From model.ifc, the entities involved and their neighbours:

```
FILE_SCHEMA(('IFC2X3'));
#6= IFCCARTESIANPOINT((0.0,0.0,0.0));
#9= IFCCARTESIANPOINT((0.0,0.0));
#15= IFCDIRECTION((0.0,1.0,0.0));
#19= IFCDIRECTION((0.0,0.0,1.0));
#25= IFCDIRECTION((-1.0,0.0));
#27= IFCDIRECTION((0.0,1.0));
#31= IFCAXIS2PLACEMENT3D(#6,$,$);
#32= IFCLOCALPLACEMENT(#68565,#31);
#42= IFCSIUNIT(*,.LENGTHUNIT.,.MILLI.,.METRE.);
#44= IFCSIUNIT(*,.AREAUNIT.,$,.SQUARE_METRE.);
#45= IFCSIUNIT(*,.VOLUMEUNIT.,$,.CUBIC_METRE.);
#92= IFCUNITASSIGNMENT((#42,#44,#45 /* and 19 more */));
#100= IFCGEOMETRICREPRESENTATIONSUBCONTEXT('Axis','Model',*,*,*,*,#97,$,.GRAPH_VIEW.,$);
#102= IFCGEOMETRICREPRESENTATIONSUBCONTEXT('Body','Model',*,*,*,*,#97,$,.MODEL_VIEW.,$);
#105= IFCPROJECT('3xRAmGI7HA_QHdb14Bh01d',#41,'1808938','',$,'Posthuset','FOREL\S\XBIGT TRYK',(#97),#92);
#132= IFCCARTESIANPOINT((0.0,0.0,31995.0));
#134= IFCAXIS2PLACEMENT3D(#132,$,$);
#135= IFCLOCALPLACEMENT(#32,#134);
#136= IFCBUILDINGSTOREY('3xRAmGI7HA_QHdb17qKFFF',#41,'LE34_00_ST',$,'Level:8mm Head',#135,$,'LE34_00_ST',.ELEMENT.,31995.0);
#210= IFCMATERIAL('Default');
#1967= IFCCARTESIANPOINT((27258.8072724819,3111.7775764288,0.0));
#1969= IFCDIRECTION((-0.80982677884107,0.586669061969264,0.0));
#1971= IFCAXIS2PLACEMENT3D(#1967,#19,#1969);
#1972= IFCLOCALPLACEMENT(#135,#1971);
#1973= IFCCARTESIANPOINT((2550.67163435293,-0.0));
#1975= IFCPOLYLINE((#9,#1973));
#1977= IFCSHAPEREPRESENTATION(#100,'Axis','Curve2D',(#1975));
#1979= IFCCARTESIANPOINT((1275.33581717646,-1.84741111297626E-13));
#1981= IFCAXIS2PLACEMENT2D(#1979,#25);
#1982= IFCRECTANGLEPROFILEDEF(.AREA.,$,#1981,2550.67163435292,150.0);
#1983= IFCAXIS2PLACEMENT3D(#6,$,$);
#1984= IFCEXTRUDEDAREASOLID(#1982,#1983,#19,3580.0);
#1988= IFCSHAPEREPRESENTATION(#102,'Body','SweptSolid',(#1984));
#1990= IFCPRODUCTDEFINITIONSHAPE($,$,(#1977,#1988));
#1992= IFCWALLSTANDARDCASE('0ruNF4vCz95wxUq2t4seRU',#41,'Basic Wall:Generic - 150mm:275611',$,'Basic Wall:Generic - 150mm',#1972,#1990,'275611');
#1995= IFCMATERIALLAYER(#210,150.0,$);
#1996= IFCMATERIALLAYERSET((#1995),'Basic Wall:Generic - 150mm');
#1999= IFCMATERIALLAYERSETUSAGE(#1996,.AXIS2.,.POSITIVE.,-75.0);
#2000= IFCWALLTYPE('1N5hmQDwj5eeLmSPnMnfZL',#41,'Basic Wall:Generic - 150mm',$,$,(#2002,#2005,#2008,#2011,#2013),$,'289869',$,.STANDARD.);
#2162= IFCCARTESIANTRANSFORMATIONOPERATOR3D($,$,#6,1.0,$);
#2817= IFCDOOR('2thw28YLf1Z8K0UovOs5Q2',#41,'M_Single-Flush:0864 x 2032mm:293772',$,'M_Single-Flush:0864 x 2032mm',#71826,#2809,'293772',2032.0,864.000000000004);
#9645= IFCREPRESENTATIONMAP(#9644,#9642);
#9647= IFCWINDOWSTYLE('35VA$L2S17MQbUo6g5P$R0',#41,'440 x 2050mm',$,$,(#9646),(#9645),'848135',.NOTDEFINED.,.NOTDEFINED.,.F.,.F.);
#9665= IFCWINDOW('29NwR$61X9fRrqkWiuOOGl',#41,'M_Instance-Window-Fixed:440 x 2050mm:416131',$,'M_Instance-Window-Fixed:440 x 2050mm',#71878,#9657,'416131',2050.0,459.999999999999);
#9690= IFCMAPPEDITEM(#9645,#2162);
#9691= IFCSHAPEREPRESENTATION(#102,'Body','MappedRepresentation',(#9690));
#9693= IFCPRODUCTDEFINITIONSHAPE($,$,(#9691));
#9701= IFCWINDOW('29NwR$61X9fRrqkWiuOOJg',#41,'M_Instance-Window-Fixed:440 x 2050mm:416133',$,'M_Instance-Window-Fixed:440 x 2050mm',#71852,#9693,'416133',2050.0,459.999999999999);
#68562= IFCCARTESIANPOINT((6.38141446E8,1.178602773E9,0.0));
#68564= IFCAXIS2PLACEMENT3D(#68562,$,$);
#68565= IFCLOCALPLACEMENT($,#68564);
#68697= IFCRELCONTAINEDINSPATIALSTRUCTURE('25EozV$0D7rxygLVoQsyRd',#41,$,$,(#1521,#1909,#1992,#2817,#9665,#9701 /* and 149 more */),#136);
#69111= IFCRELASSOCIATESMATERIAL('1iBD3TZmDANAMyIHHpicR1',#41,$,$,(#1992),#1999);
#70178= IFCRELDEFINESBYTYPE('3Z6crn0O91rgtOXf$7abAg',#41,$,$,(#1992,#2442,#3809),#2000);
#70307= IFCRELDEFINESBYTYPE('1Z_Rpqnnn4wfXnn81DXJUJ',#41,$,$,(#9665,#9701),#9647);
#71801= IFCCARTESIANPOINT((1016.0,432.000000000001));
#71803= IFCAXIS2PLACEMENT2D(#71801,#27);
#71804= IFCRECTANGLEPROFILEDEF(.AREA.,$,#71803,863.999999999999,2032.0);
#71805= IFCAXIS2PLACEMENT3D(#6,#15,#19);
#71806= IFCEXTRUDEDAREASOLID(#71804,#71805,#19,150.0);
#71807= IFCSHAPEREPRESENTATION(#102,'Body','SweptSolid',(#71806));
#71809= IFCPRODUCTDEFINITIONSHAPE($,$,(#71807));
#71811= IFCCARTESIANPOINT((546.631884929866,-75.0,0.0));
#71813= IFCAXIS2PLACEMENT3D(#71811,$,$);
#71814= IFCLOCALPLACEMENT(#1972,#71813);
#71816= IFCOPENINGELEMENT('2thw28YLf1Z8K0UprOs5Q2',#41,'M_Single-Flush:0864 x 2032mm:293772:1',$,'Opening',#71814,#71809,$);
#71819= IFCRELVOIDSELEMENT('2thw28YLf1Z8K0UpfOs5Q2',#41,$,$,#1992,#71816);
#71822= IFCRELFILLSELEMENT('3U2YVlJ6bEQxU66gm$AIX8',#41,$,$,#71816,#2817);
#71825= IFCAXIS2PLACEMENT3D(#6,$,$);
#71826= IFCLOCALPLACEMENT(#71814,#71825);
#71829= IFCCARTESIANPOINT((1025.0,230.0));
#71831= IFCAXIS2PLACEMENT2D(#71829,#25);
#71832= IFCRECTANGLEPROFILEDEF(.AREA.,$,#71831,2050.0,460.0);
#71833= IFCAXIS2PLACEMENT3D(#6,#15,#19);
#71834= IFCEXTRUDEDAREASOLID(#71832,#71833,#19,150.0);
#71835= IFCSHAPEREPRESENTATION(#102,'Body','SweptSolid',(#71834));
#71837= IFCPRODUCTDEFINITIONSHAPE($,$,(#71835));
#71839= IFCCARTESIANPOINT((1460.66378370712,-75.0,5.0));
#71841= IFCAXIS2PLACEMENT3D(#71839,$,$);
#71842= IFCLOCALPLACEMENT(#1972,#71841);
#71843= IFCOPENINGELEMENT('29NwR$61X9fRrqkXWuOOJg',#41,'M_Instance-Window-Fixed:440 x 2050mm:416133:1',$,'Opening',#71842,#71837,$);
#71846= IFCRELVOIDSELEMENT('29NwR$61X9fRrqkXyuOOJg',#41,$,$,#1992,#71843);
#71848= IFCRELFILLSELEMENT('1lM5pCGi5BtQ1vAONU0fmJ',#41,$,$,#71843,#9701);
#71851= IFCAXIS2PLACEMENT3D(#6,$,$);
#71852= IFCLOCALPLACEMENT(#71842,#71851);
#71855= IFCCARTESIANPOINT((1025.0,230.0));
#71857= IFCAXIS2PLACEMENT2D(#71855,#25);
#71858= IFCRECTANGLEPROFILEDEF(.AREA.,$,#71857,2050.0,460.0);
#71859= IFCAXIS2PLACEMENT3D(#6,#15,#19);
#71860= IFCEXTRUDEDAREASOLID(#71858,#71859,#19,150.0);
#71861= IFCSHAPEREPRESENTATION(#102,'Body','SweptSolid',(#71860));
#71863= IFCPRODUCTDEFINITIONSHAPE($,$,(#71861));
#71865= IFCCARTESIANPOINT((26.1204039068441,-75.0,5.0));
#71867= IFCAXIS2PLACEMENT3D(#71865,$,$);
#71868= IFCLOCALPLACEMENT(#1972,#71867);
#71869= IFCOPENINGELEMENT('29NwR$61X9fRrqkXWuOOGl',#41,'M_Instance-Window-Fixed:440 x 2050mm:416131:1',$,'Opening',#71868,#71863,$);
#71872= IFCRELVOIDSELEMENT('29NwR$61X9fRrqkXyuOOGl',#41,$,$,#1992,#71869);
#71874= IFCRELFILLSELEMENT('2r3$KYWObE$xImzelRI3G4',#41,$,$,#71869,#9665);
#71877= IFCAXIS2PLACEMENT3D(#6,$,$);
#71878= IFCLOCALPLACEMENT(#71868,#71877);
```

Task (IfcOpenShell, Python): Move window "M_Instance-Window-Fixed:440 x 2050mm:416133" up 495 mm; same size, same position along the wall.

```python
import numpy as np
import ifcopenshell
import ifcopenshell.api.geometry
import ifcopenshell.util.placement
import ifcopenshell.util.unit

model = ifcopenshell.open("model.ifc")
unit_scale = ifcopenshell.util.unit.calculate_unit_scale(model)

window = model.by_guid("29NwR$61X9fRrqkWiuOOJg")
opening = window.FillsVoids[0].RelatingOpeningElement
dz = 495.0

shift = np.array([0.0, 0.0, dz])
# The window is placed relative to its opening, so it follows when the opening moves.
matrix = ifcopenshell.util.placement.get_local_placement(opening.ObjectPlacement)
matrix[:3, 3] += shift
ifcopenshell.api.geometry.edit_object_placement(
    model, product=opening, matrix=matrix, is_si=False, should_transform_children=True
)

print(f"moved by {dz * unit_scale:+.3f} m")

model.write("model-out.ifc")
```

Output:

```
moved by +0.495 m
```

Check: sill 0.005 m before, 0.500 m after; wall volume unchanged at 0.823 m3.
